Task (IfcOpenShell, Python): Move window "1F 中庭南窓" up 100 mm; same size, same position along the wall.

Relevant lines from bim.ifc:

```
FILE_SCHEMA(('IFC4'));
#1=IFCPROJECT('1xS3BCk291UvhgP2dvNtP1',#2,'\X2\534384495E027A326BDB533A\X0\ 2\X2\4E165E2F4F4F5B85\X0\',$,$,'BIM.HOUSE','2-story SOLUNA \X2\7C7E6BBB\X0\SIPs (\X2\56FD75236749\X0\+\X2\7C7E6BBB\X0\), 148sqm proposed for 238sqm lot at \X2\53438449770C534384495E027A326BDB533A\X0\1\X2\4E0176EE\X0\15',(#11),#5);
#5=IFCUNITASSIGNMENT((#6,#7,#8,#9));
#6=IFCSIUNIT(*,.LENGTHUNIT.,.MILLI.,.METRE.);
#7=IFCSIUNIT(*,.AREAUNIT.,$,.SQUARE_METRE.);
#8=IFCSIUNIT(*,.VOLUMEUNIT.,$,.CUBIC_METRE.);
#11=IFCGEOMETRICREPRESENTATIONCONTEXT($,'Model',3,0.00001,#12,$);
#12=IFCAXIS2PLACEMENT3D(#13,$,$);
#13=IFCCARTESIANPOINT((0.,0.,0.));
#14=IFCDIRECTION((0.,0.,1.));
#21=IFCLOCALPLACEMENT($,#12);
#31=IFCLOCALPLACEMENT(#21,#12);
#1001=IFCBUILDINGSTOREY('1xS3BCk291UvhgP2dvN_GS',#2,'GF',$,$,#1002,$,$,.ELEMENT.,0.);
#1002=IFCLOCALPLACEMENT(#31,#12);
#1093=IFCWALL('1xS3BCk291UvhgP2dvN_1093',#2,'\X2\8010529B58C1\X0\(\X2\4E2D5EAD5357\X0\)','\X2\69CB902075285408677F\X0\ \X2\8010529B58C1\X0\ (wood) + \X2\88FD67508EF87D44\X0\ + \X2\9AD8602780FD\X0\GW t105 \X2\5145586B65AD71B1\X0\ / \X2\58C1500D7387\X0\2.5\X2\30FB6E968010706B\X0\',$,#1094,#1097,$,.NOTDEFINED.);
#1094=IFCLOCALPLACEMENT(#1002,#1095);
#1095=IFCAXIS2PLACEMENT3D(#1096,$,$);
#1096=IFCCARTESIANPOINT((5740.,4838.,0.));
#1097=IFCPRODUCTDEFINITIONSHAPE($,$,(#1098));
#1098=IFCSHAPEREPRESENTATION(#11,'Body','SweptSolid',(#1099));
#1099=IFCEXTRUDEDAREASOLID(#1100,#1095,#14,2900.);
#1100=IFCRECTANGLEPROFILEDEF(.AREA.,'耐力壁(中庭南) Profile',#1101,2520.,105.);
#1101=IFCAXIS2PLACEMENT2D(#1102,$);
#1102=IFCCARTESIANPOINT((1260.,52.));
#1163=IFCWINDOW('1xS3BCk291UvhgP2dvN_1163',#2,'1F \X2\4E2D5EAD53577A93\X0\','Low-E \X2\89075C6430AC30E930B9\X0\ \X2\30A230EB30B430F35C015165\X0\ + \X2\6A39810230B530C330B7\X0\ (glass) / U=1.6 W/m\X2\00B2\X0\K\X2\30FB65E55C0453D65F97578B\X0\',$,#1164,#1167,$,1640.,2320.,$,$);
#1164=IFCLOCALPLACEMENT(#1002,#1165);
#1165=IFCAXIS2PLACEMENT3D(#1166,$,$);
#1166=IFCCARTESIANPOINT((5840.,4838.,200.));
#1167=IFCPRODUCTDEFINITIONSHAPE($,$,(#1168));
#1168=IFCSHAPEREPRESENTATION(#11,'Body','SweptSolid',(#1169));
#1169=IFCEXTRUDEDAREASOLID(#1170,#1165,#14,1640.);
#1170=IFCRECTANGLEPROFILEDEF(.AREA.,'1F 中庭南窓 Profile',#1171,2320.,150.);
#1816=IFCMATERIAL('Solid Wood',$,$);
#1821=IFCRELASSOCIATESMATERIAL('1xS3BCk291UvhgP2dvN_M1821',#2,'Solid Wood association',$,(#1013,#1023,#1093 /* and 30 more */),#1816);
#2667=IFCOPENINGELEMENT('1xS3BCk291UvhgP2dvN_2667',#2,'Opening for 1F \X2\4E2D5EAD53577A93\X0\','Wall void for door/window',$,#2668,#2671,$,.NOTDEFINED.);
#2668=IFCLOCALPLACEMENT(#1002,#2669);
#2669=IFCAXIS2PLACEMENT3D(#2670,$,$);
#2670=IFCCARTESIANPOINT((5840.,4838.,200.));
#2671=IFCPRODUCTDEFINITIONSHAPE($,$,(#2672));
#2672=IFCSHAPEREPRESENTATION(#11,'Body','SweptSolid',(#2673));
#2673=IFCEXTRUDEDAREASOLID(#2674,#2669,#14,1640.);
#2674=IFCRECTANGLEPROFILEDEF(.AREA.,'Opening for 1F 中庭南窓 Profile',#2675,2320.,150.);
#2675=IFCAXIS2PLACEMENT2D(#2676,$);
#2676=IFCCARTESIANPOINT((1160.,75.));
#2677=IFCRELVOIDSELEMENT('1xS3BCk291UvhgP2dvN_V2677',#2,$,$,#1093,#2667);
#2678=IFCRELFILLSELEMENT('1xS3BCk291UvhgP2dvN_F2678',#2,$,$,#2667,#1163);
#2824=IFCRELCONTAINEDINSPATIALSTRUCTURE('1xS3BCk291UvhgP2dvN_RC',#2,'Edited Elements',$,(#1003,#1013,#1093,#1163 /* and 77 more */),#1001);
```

```python
import numpy as np
import ifcopenshell
import ifcopenshell.api.geometry
import ifcopenshell.util.placement
import ifcopenshell.util.unit

model = ifcopenshell.open("bim.ifc")
unit_scale = ifcopenshell.util.unit.calculate_unit_scale(model)

window = model.by_guid("1xS3BCk291UvhgP2dvN_1163")
opening = window.FillsVoids[0].RelatingOpeningElement
dz = 0.1 / unit_scale

shift = np.array([0.0, 0.0, dz])
# The window is not placed relative to its opening, so move both.
for product in (opening, window):
    matrix = ifcopenshell.util.placement.get_local_placement(product.ObjectPlacement)
    matrix[:3, 3] += shift
    ifcopenshell.api.geometry.edit_object_placement(model, product=product, matrix=matrix, is_si=False)

print(f"moved by {dz * unit_scale:+.3f} m")

model.write("bim_updated.ifc")
```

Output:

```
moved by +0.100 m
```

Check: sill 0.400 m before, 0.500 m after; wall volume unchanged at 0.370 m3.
